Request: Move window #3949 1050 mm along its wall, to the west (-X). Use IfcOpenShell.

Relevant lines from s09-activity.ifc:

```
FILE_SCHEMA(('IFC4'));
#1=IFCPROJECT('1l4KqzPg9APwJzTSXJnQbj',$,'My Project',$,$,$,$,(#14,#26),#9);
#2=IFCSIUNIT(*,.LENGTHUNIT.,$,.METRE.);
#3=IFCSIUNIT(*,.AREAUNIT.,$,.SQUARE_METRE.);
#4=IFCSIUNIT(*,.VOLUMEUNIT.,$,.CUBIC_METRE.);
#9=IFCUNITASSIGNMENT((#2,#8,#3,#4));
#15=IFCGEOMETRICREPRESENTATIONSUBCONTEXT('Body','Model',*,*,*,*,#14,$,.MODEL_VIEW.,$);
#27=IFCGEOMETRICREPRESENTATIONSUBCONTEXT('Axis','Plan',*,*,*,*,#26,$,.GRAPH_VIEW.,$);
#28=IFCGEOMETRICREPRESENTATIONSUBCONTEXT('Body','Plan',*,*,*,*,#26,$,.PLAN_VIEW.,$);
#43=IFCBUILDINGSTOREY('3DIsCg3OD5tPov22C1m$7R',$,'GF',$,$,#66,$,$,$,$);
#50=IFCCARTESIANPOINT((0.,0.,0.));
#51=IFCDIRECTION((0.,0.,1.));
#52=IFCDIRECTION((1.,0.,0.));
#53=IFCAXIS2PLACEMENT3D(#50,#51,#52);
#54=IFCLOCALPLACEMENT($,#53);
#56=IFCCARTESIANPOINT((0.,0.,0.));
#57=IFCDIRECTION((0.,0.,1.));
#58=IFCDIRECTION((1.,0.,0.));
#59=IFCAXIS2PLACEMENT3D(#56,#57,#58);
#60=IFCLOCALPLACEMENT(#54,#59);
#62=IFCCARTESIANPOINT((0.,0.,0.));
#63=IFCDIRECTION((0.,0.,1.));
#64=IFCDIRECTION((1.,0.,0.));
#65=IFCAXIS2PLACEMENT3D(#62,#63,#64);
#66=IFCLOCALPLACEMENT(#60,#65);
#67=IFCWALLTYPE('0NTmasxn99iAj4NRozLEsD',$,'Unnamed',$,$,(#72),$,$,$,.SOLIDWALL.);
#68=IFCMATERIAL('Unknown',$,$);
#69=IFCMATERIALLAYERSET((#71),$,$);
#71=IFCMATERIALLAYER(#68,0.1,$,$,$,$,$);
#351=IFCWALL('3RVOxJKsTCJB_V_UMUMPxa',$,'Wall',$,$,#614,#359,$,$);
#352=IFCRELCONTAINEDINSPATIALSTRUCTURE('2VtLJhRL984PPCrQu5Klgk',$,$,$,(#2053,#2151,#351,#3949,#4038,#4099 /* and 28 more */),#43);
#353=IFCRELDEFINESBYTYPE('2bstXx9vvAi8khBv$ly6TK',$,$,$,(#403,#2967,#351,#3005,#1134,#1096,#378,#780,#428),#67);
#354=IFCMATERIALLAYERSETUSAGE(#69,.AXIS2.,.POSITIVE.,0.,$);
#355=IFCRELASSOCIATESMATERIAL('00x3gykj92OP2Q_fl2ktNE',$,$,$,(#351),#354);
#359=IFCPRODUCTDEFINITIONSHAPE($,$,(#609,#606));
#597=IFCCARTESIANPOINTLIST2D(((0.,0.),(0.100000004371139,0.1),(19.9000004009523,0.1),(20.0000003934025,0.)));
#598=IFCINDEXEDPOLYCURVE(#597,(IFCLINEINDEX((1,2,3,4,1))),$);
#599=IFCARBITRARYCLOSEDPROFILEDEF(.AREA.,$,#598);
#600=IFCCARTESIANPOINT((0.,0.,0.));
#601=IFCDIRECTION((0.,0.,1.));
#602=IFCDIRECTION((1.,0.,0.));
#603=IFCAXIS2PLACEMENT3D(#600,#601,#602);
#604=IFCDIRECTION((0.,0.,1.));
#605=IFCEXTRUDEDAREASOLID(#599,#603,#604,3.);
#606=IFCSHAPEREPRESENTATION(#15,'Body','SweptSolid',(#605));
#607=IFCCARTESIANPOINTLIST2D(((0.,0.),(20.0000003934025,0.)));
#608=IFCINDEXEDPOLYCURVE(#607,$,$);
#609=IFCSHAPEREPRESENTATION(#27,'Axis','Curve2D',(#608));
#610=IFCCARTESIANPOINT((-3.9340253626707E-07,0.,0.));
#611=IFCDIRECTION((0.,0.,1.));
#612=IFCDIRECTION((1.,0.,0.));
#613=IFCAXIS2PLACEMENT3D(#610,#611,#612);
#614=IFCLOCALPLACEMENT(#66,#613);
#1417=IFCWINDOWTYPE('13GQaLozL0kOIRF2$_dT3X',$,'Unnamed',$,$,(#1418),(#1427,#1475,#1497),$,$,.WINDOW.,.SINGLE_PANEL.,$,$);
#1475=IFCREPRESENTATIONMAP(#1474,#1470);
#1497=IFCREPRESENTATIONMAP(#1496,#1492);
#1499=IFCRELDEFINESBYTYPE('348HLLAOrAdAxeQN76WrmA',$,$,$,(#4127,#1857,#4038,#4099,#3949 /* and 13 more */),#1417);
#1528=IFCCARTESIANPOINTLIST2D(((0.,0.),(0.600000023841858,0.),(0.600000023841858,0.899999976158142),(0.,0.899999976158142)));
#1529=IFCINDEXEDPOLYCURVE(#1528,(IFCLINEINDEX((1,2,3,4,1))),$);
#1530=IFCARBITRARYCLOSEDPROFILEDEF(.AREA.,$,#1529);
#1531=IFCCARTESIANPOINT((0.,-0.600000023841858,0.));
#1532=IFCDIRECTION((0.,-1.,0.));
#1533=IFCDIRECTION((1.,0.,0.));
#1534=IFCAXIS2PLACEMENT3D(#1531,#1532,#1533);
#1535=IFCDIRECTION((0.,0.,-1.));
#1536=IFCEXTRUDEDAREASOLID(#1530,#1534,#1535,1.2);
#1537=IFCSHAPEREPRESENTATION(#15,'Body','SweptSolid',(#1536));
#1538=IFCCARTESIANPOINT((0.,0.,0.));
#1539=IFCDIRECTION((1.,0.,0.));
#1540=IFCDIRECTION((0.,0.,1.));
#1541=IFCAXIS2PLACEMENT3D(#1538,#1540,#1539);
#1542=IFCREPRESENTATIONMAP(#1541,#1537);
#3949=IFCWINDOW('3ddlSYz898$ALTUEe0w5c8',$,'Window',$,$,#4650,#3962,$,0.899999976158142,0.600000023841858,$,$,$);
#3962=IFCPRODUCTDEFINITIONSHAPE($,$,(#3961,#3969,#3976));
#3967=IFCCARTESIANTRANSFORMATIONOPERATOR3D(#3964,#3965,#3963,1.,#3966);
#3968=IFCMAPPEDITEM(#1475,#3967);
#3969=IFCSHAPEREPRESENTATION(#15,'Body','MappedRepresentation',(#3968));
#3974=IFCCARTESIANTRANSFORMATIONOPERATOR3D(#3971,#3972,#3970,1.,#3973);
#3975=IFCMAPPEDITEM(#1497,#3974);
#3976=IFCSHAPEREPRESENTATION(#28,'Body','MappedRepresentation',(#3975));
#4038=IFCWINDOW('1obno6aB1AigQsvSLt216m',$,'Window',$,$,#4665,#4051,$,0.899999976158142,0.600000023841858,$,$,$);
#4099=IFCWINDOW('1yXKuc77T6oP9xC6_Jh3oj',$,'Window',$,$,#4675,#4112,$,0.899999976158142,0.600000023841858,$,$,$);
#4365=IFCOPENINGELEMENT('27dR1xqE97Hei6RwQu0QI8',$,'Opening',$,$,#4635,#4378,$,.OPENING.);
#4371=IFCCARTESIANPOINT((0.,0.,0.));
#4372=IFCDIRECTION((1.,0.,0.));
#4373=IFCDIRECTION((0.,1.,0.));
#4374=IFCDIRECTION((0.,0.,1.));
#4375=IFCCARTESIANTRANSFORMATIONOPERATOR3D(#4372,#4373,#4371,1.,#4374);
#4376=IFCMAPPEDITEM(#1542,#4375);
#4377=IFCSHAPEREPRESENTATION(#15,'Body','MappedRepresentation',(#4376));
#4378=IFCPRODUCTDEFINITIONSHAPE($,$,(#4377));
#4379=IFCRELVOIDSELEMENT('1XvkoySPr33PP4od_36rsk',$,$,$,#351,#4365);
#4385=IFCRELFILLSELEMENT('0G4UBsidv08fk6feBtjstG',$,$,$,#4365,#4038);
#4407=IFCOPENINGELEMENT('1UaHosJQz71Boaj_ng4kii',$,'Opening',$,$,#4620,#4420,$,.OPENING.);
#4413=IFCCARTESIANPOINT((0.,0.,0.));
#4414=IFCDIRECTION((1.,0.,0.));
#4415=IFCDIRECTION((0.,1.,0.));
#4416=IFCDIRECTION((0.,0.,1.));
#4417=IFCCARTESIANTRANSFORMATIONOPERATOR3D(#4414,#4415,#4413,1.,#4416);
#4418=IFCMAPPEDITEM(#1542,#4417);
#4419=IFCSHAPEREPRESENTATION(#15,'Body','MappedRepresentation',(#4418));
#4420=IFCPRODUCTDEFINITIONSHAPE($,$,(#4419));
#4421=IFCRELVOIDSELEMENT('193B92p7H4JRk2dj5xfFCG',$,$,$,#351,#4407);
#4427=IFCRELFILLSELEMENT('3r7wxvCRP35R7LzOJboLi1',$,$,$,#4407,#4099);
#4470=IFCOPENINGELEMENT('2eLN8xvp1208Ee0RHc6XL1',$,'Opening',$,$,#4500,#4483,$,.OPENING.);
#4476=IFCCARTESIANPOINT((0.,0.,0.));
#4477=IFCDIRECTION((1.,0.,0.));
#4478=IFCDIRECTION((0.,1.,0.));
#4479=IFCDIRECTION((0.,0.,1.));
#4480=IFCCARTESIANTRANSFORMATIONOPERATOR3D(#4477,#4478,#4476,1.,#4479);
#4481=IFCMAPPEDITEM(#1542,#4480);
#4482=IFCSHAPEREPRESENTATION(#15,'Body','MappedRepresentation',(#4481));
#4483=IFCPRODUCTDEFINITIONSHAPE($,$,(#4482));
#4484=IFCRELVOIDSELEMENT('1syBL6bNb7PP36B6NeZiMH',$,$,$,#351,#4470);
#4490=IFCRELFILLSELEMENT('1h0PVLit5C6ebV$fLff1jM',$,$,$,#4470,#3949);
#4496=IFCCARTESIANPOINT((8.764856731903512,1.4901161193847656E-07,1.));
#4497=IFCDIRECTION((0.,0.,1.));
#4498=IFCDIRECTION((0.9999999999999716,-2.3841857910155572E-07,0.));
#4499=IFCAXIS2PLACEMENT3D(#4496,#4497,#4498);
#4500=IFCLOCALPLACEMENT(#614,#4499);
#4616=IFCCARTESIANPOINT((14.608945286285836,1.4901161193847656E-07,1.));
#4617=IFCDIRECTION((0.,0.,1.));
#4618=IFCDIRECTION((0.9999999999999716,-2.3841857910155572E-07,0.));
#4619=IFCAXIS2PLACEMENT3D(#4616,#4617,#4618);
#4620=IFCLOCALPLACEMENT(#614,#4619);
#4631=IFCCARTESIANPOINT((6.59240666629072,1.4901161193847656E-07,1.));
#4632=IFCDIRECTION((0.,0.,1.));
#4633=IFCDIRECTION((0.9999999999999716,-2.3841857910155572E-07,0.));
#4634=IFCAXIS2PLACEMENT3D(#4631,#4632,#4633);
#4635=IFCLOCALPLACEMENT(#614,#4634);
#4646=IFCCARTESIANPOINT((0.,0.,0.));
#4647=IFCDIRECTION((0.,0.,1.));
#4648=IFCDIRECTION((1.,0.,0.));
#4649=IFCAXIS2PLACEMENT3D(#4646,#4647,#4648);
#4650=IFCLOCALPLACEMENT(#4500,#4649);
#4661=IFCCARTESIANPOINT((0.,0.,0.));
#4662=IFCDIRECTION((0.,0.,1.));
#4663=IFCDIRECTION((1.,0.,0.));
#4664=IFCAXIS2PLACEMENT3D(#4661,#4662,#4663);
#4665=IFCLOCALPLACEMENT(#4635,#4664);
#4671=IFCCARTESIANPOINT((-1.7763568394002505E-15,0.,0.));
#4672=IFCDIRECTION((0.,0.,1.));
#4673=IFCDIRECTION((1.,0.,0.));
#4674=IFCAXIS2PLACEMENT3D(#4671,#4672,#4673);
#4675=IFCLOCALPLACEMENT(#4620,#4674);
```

```python
import ifcopenshell
import ifcopenshell.api.geometry
import ifcopenshell.util.placement
import ifcopenshell.util.unit

model = ifcopenshell.open("s09-activity.ifc")
unit_scale = ifcopenshell.util.unit.calculate_unit_scale(model)

window = model.by_id(3949)
opening = window.FillsVoids[0].RelatingOpeningElement
wall = opening.VoidsElements[0].RelatingBuildingElement

wall_matrix = ifcopenshell.util.placement.get_local_placement(wall.ObjectPlacement)
shift = wall_matrix[:3, 0] * -1.05 / unit_scale
before = ifcopenshell.util.placement.get_local_placement(window.ObjectPlacement)[:3, 3].copy()

# The window is placed relative to its opening, so it follows when the opening moves.
matrix = ifcopenshell.util.placement.get_local_placement(opening.ObjectPlacement)
matrix[:3, 3] += shift
ifcopenshell.api.geometry.edit_object_placement(
    model, product=opening, matrix=matrix, is_si=False, should_transform_children=True
)

after = ifcopenshell.util.placement.get_local_placement(window.ObjectPlacement)[:3, 3]
print("window moved by", (after - before).round(3) + 0.0)

model.write("s09-activity-out.ifc")
```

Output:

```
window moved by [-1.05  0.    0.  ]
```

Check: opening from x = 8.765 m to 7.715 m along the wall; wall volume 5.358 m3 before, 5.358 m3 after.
